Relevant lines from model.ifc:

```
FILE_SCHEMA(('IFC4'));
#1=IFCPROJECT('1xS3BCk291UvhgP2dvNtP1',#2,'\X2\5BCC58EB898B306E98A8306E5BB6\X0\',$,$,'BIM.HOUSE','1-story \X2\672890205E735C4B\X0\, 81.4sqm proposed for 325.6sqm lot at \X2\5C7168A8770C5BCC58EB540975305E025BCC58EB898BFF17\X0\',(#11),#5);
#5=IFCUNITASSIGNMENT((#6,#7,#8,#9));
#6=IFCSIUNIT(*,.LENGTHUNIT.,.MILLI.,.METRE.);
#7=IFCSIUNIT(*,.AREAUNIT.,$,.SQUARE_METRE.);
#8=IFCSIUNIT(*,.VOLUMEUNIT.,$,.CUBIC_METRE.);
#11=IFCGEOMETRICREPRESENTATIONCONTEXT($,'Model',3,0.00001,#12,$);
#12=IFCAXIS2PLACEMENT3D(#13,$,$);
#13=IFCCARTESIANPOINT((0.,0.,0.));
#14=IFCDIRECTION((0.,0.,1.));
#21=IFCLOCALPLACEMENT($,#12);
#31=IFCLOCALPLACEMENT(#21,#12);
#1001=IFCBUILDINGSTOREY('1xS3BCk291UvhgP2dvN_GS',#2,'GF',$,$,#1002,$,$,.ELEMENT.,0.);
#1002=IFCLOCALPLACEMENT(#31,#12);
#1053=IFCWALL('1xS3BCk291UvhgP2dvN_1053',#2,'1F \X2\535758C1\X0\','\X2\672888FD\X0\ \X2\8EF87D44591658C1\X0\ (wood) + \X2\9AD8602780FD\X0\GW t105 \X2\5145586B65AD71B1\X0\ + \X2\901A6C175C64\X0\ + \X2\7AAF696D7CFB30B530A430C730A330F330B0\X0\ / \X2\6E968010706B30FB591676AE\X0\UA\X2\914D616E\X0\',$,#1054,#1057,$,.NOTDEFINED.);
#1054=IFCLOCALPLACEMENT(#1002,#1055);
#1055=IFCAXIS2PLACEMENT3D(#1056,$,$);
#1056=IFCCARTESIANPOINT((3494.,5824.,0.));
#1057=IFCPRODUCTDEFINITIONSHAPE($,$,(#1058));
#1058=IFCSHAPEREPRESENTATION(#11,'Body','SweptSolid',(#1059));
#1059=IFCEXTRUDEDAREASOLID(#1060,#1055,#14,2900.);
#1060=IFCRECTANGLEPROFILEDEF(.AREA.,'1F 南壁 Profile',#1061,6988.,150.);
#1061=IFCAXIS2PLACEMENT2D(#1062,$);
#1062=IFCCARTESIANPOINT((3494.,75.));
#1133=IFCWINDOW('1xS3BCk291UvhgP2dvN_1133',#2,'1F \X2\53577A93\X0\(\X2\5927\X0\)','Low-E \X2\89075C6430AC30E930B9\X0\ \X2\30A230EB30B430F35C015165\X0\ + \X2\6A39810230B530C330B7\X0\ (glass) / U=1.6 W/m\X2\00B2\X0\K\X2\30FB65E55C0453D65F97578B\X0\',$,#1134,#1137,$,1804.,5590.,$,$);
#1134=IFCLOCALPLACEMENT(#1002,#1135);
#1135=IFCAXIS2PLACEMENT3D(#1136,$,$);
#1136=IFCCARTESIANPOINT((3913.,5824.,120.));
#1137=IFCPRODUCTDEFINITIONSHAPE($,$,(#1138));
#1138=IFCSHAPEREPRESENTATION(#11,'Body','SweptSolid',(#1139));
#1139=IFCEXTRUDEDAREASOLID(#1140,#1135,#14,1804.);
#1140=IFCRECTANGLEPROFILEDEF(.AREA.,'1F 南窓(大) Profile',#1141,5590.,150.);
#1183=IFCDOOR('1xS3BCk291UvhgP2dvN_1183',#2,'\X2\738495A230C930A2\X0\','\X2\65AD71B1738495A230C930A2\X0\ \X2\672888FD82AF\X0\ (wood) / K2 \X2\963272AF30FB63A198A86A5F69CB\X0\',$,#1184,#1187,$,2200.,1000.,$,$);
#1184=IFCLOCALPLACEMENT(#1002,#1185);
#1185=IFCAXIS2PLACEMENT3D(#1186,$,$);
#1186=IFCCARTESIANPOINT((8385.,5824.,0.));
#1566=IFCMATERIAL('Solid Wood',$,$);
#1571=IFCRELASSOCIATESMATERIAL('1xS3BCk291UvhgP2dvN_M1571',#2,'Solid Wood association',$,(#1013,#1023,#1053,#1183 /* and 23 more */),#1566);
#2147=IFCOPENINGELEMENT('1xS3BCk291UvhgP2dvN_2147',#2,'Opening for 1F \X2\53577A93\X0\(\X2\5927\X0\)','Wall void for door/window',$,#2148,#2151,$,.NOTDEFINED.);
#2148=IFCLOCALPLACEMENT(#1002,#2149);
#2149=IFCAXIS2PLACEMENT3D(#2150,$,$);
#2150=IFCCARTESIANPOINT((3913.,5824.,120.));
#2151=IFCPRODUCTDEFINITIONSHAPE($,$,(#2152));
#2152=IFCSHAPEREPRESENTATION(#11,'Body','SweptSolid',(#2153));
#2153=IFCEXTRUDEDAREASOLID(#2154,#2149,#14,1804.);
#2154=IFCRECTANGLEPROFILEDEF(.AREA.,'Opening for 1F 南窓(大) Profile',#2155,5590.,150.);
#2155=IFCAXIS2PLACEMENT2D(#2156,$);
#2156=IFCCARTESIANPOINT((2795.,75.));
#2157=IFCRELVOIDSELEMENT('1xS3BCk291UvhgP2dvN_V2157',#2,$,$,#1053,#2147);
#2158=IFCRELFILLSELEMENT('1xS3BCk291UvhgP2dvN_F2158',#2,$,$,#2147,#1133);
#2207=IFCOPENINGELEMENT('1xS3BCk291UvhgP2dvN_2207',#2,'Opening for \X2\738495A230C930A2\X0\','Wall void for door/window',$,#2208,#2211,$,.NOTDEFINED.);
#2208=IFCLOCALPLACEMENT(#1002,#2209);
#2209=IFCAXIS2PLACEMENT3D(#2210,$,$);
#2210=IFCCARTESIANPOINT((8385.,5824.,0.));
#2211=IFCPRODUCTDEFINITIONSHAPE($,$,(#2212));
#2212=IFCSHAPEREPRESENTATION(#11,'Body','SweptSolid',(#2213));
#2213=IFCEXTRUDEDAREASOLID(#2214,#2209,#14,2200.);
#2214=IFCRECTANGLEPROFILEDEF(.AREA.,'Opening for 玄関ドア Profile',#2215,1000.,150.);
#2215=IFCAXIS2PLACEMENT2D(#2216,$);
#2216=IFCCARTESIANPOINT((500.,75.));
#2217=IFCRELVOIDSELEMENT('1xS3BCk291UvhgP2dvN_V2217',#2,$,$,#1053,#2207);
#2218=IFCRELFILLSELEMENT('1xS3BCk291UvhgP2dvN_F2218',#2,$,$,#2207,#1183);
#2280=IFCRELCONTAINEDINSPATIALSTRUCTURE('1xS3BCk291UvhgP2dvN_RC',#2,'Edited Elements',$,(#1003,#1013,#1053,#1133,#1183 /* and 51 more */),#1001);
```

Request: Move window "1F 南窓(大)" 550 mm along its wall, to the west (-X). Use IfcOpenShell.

```python
import ifcopenshell
import ifcopenshell.api.geometry
import ifcopenshell.util.placement
import ifcopenshell.util.unit

model = ifcopenshell.open("model.ifc")
unit_scale = ifcopenshell.util.unit.calculate_unit_scale(model)

window = model.by_guid("1xS3BCk291UvhgP2dvN_1133")
opening = window.FillsVoids[0].RelatingOpeningElement
wall = opening.VoidsElements[0].RelatingBuildingElement

wall_matrix = ifcopenshell.util.placement.get_local_placement(wall.ObjectPlacement)
shift = wall_matrix[:3, 0] * -0.55 / unit_scale
before = ifcopenshell.util.placement.get_local_placement(window.ObjectPlacement)[:3, 3].copy()

# The window is not placed relative to its opening, so move both.
for product in (opening, window):
    matrix = ifcopenshell.util.placement.get_local_placement(product.ObjectPlacement)
    matrix[:3, 3] += shift
    ifcopenshell.api.geometry.edit_object_placement(model, product=product, matrix=matrix, is_si=False)

after = ifcopenshell.util.placement.get_local_placement(window.ObjectPlacement)[:3, 3]
print("window moved by", (after - before).round(3) + 0.0)

model.write("model_rev.ifc")
```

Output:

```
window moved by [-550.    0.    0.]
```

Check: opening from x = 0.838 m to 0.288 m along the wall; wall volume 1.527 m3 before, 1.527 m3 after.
